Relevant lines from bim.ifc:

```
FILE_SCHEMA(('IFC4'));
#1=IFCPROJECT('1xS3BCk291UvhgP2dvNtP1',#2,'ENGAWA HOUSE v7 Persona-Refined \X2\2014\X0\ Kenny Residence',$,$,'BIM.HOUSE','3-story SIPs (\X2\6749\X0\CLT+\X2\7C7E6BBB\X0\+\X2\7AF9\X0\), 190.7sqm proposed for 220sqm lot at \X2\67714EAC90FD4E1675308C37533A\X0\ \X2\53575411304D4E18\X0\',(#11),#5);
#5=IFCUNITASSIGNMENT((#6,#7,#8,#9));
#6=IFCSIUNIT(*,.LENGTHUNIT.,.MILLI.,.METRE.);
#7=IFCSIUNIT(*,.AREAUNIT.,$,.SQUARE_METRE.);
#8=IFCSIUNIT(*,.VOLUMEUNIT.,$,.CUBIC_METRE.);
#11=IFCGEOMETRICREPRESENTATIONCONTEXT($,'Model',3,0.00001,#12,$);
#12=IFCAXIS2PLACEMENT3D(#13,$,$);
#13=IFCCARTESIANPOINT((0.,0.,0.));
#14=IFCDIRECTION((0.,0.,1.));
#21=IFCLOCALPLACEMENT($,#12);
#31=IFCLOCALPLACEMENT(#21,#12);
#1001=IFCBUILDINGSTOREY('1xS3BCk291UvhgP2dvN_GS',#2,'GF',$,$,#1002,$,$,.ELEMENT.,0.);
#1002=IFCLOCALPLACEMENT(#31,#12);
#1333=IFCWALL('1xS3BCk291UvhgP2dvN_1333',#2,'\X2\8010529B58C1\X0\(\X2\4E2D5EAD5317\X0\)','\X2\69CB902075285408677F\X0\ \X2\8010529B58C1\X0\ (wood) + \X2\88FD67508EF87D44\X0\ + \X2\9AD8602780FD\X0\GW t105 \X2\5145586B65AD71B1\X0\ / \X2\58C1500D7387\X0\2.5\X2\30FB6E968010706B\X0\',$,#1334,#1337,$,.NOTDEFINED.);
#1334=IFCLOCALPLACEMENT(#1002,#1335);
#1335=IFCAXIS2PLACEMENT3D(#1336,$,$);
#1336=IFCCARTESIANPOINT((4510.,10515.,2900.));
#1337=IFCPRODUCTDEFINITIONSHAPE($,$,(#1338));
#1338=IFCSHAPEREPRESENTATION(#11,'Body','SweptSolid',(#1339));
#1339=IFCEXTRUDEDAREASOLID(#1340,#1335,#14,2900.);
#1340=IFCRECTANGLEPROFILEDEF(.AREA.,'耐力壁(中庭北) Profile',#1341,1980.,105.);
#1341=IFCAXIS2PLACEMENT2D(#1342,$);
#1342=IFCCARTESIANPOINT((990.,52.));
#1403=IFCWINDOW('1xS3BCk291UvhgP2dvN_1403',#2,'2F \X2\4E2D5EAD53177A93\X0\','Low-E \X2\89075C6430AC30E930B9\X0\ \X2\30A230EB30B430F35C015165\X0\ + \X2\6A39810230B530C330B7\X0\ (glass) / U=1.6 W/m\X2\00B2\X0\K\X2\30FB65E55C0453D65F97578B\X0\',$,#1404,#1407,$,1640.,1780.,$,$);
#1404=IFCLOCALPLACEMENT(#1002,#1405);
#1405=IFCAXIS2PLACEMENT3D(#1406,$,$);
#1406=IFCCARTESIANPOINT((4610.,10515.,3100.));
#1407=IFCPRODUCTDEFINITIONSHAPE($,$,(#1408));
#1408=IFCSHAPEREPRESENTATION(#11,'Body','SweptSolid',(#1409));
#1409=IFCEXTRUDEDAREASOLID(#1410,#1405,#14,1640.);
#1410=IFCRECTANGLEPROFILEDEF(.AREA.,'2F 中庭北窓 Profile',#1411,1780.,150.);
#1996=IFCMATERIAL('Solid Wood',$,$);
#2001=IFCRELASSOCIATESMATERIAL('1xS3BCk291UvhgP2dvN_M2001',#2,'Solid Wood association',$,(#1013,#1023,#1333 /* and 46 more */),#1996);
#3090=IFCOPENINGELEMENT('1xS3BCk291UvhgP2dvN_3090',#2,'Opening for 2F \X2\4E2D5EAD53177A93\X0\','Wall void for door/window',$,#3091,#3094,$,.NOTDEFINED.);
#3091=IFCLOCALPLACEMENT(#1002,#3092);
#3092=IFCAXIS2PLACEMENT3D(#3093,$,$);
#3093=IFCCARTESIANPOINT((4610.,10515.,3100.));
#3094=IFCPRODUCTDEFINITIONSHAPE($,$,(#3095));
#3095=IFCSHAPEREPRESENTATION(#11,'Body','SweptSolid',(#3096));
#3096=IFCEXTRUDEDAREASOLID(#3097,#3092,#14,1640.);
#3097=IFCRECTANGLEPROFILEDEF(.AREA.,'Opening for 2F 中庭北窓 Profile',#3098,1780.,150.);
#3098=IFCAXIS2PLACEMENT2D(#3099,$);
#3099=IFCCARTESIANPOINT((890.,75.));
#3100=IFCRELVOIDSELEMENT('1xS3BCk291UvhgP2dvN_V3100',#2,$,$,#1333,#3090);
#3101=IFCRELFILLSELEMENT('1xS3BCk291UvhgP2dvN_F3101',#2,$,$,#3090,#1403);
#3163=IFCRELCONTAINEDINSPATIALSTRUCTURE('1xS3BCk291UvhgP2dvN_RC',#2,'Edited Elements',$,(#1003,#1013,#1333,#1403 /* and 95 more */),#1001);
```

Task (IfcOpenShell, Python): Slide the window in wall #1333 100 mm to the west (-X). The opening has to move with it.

```python
import ifcopenshell
import ifcopenshell.api.geometry
import ifcopenshell.util.placement
import ifcopenshell.util.unit

model = ifcopenshell.open("bim.ifc")
unit_scale = ifcopenshell.util.unit.calculate_unit_scale(model)

window = model.by_id(1403)
opening = window.FillsVoids[0].RelatingOpeningElement
wall = opening.VoidsElements[0].RelatingBuildingElement

wall_matrix = ifcopenshell.util.placement.get_local_placement(wall.ObjectPlacement)
shift = wall_matrix[:3, 0] * -0.1 / unit_scale
before = ifcopenshell.util.placement.get_local_placement(window.ObjectPlacement)[:3, 3].copy()

# The window is not placed relative to its opening, so move both.
for product in (opening, window):
    matrix = ifcopenshell.util.placement.get_local_placement(product.ObjectPlacement)
    matrix[:3, 3] += shift
    ifcopenshell.api.geometry.edit_object_placement(model, product=product, matrix=matrix, is_si=False)

after = ifcopenshell.util.placement.get_local_placement(window.ObjectPlacement)[:3, 3]
print("window moved by", (after - before).round(3) + 0.0)

model.write("bim_rev.ifc")
```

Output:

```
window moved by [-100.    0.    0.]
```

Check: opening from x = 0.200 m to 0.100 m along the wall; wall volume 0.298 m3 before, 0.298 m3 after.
